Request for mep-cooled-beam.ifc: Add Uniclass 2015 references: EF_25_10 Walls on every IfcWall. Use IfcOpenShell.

First a look at what the model holds.

```python
import ifcopenshell

model = ifcopenshell.open("mep-cooled-beam.ifc")
print(model.schema)
print("classifications:", [c.Name for c in model.by_type("IfcClassification")])
for ifc_class in ("IfcDoor", "IfcRoof", "IfcStair", "IfcWall", "IfcWindow"):
    print(ifc_class, len(model.by_type(ifc_class)))
```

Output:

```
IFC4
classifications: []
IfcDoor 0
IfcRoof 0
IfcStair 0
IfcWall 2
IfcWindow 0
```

```python
import ifcopenshell
import ifcopenshell.api.classification

model = ifcopenshell.open("mep-cooled-beam.ifc")

system = ifcopenshell.api.classification.add_classification(model, classification="Uniclass 2015")

codes = {
    "IfcWall": ("EF_25_10", "Walls"),
}
for ifc_class, (code, name) in codes.items():
    products = model.by_type(ifc_class)
    ifcopenshell.api.classification.add_reference(
        model, products=products, classification=system, identification=code, name=name
    )
    print(code, len(products))

model.write("mep-cooled-beam-out.ifc")
```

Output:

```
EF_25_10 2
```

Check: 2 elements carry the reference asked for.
